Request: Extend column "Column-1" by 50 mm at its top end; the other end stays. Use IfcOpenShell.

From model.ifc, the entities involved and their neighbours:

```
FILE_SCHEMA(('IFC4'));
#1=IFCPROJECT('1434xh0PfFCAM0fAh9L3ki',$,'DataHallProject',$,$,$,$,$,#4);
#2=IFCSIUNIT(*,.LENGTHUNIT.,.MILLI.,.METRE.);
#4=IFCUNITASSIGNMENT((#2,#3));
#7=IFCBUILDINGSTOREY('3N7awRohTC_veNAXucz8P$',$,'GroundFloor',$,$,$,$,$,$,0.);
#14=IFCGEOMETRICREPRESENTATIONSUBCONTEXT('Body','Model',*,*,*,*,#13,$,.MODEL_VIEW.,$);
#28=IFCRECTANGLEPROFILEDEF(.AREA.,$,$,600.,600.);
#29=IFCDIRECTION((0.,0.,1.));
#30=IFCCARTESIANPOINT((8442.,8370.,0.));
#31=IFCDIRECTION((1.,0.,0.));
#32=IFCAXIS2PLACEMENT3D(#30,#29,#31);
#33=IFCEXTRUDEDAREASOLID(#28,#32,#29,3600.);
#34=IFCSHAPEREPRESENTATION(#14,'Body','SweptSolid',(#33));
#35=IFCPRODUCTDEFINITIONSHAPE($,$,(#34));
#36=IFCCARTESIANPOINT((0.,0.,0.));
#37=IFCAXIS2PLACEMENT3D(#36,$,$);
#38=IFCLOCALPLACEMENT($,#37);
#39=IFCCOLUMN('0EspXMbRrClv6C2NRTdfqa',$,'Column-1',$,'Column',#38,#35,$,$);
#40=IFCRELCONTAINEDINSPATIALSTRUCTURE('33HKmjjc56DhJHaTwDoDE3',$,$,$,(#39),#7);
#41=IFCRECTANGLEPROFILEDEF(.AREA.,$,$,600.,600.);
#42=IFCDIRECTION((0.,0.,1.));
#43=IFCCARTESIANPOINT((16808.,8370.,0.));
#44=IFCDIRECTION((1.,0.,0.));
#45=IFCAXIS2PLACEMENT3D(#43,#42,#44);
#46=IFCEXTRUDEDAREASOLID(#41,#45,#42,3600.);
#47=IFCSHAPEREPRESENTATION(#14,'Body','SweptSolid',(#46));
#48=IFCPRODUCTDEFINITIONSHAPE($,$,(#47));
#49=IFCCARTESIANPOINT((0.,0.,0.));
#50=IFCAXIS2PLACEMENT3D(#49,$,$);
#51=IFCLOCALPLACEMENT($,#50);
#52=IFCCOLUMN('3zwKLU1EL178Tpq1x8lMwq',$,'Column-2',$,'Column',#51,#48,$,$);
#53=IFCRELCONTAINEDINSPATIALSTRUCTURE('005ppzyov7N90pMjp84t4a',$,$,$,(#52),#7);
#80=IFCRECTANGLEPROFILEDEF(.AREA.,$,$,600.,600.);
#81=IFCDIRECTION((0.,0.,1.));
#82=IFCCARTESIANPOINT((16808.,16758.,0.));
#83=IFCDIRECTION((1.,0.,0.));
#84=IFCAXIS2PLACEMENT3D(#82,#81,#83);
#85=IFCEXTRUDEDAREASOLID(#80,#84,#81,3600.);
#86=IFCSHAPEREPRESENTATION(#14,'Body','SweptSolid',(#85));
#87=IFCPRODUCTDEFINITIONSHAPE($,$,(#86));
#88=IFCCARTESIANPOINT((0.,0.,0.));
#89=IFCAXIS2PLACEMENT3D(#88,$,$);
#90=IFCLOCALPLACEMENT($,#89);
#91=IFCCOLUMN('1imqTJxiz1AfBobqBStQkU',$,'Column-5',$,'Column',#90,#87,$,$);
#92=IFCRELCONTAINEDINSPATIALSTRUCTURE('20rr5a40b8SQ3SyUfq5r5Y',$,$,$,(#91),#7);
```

```python
import ifcopenshell
import ifcopenshell.util.representation

model = ifcopenshell.open("model.ifc")

member = model.by_guid("0EspXMbRrClv6C2NRTdfqa")
change = 50.0

# The extrusion runs towards the end named, so only its depth changes.
body = ifcopenshell.util.representation.get_representation(member, "Model", "Body")
solid = body.Items[0]
old_length = solid.Depth
solid.Depth += change

print(f"length {old_length:g} -> {solid.Depth:g}")

model.write("model_rev.ifc")
```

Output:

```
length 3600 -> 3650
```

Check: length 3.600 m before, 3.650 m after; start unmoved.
